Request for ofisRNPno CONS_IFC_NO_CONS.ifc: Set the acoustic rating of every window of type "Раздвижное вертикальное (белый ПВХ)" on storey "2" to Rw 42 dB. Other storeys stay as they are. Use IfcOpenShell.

First a look at what the model holds.

```python
import ifcopenshell
import ifcopenshell.util.element

model = ifcopenshell.open("ofisRNPno CONS_IFC_NO_CONS.ifc")
print(model.schema)
storey = next(s for s in model.by_type("IfcBuildingStorey") if s.Name == "2")
windows = [e for e in ifcopenshell.util.element.get_decomposition(storey) if e.is_a("IfcWindow")]
seen = {}
for e in windows:
    element_type = ifcopenshell.util.element.get_type(e)
    key = (element_type.Name if element_type != e and element_type else None, ifcopenshell.util.element.get_pset(e, "Pset_WindowCommon", "AcousticRating"))
    seen[key] = seen.get(key, 0) + 1
for (name, value), count in sorted(seen.items(), key=str):
    print(count, "x", name, "|", value)
```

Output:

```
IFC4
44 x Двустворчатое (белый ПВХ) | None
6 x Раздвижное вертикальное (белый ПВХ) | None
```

```python
import ifcopenshell
import ifcopenshell.api.pset
import ifcopenshell.util.element

model = ifcopenshell.open("ofisRNPno CONS_IFC_NO_CONS.ifc")

storey = next(s for s in model.by_type("IfcBuildingStorey") if s.Name == "2")
windows = [e for e in ifcopenshell.util.element.get_decomposition(storey) if e.is_a("IfcWindow")]

count = 0
for e in windows:
    element_type = ifcopenshell.util.element.get_type(e)
    if element_type in (None, e) or element_type.Name != "Раздвижное вертикальное (белый ПВХ)":
        continue
    # add_pset returns the element's existing set when there is one.
    pset = ifcopenshell.api.pset.add_pset(model, product=e, name="Pset_WindowCommon")
    ifcopenshell.api.pset.edit_pset(model, pset=pset, properties={"AcousticRating": "Rw 42 dB"})
    count += 1

print(count, "windows updated")

model.write("ofisRNPno CONS_IFC_NO_CONS_rev.ifc")
```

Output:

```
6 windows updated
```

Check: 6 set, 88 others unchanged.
